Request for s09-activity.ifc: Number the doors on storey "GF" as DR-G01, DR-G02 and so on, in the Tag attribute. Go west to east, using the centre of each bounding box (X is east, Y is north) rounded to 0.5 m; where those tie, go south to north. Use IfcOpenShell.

First a look at what the model holds.

```python
import ifcopenshell
import ifcopenshell.util.element
import ifcopenshell.util.placement

model = ifcopenshell.open("s09-activity.ifc")
print(model.schema)
storey = next(s for s in model.by_type("IfcBuildingStorey") if s.Name == "GF")
doors = [e for e in ifcopenshell.util.element.get_decomposition(storey) if e.is_a("IfcDoor")]
for e in sorted(doors, key=lambda e: e.id()):
    origin = ifcopenshell.util.placement.get_local_placement(e.ObjectPlacement)[:3, 3]
    print(e.id(), e.Tag, e.Name, origin.round(2) + 0.0, sep=" | ")
```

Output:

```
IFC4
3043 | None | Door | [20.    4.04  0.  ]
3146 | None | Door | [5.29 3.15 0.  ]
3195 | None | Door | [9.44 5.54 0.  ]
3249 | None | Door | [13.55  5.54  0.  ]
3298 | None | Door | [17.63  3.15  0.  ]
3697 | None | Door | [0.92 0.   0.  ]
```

```python
import ifcopenshell
import ifcopenshell.geom
import ifcopenshell.util.element
import ifcopenshell.util.shape

model = ifcopenshell.open("s09-activity.ifc")
settings = ifcopenshell.geom.settings()
settings.set("use-world-coords", True)


def centre(element):
    shape = ifcopenshell.geom.create_shape(settings, element)
    return ifcopenshell.util.shape.get_bbox_centroid(shape.geometry)


storey = next(s for s in model.by_type("IfcBuildingStorey") if s.Name == "GF")
doors = [e for e in ifcopenshell.util.element.get_decomposition(storey) if e.is_a("IfcDoor")]

# Insertion points can sit at a corner or the storey origin, so sort by the geometry (in metres).
centres = {e: centre(e) for e in doors}
doors.sort(key=lambda e: (round(centres[e][0] / 0.5), centres[e][1]))

for i, e in enumerate(doors, start=1):
    number = f"DR-G{i:02d}"
    e.Tag = number
    print(e.id(), number)

model.write("s09-activity_rev.ifc")
```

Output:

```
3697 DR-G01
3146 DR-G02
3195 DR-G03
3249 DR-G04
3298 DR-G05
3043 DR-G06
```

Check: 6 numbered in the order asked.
